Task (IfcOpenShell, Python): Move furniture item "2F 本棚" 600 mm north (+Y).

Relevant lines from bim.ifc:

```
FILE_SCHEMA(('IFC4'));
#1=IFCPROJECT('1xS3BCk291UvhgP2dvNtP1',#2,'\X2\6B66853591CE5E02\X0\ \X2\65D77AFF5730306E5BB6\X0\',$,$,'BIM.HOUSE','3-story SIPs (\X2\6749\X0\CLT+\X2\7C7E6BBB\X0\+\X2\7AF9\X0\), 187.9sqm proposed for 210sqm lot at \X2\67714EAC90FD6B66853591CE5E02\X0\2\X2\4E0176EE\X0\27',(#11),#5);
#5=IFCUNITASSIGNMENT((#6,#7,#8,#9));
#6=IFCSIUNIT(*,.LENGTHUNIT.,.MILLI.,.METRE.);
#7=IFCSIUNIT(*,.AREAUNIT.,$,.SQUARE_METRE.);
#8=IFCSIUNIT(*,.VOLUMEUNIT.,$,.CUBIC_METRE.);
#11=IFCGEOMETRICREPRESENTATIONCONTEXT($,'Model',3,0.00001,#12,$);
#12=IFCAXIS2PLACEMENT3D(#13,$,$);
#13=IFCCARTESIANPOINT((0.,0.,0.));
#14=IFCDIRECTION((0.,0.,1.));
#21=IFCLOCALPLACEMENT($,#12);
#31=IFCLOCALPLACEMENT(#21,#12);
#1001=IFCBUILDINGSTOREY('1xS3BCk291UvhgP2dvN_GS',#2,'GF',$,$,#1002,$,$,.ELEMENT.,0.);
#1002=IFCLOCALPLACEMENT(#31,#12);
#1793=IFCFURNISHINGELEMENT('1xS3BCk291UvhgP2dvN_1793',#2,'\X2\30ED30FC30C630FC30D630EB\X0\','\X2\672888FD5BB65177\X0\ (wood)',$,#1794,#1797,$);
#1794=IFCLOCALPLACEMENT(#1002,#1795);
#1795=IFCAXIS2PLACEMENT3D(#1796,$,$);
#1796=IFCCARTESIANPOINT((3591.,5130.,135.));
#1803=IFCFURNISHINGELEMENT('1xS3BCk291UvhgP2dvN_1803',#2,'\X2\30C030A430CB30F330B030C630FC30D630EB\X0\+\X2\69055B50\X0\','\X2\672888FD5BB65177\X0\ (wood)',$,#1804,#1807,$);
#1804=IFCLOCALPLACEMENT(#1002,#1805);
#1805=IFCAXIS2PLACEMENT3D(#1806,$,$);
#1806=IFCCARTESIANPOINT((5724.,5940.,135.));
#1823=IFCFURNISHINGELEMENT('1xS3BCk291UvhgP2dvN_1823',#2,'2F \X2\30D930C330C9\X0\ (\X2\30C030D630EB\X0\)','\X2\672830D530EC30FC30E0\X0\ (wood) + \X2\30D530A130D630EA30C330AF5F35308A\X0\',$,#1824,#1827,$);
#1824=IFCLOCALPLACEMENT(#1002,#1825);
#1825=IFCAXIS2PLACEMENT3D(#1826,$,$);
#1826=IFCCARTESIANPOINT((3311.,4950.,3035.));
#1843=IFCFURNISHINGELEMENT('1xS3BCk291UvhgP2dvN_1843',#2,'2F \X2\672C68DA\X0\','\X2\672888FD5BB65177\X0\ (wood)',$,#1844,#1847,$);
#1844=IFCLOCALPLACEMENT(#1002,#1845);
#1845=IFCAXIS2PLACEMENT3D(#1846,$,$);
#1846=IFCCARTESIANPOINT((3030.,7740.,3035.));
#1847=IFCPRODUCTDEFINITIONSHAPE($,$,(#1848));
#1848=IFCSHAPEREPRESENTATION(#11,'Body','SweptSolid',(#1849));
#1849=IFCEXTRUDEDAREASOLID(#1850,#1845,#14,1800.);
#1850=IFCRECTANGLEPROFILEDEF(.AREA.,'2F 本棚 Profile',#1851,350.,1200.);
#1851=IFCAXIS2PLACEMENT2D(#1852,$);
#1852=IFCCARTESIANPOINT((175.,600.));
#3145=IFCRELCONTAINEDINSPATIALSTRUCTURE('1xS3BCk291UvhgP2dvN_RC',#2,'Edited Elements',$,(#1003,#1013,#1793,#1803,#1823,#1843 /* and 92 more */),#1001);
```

```python
import ifcopenshell
import ifcopenshell.api.geometry
import ifcopenshell.util.placement

model = ifcopenshell.open("bim.ifc")

item = model.by_guid("1xS3BCk291UvhgP2dvN_1843")
matrix = ifcopenshell.util.placement.get_local_placement(item.ObjectPlacement)
matrix[1, 3] += 600.0
ifcopenshell.api.geometry.edit_object_placement(model, product=item, matrix=matrix, is_si=False)

print(ifcopenshell.util.placement.get_local_placement(item.ObjectPlacement).round(3) + 0.0)

model.write("bim_rev.ifc")
```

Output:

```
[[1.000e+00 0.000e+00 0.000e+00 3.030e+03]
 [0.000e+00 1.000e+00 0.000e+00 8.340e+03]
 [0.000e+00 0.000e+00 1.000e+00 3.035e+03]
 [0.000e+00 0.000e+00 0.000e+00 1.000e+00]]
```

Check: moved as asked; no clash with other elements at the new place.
